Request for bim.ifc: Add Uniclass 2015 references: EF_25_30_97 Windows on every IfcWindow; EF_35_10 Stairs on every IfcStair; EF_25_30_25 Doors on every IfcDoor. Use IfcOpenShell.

First a look at what the model holds.

```python
import ifcopenshell

model = ifcopenshell.open("bim.ifc")
print(model.schema)
print("classifications:", [c.Name for c in model.by_type("IfcClassification")])
for ifc_class in ("IfcDoor", "IfcRoof", "IfcStair", "IfcWall", "IfcWindow"):
    print(ifc_class, len(model.by_type(ifc_class)))
```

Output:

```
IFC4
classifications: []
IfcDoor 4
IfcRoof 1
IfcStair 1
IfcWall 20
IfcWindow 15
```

```python
import ifcopenshell
import ifcopenshell.api.classification

model = ifcopenshell.open("bim.ifc")

system = ifcopenshell.api.classification.add_classification(model, classification="Uniclass 2015")

codes = {
    "IfcWindow": ("EF_25_30_97", "Windows"),
    "IfcStair": ("EF_35_10", "Stairs"),
    "IfcDoor": ("EF_25_30_25", "Doors"),
}
for ifc_class, (code, name) in codes.items():
    products = model.by_type(ifc_class)
    ifcopenshell.api.classification.add_reference(
        model, products=products, classification=system, identification=code, name=name
    )
    print(code, len(products))

model.write("bim_edited.ifc")
```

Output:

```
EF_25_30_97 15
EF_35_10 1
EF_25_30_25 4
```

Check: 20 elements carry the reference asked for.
